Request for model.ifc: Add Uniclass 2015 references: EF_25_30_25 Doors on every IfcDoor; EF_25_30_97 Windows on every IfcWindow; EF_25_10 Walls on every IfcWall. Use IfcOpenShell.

First a look at what the model holds.

```python
import ifcopenshell

model = ifcopenshell.open("model.ifc")
print(model.schema)
print("classifications:", [c.Name for c in model.by_type("IfcClassification")])
for ifc_class in ("IfcDoor", "IfcRoof", "IfcStair", "IfcWall", "IfcWindow"):
    print(ifc_class, len(model.by_type(ifc_class)))
```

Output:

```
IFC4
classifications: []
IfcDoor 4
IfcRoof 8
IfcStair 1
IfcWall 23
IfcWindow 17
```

```python
import ifcopenshell
import ifcopenshell.api.classification

model = ifcopenshell.open("model.ifc")

system = ifcopenshell.api.classification.add_classification(model, classification="Uniclass 2015")

codes = {
    "IfcDoor": ("EF_25_30_25", "Doors"),
    "IfcWindow": ("EF_25_30_97", "Windows"),
    "IfcWall": ("EF_25_10", "Walls"),
}
for ifc_class, (code, name) in codes.items():
    products = model.by_type(ifc_class)
    ifcopenshell.api.classification.add_reference(
        model, products=products, classification=system, identification=code, name=name
    )
    print(code, len(products))

model.write("model_edited.ifc")
```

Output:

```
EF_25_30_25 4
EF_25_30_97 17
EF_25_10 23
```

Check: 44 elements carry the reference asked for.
